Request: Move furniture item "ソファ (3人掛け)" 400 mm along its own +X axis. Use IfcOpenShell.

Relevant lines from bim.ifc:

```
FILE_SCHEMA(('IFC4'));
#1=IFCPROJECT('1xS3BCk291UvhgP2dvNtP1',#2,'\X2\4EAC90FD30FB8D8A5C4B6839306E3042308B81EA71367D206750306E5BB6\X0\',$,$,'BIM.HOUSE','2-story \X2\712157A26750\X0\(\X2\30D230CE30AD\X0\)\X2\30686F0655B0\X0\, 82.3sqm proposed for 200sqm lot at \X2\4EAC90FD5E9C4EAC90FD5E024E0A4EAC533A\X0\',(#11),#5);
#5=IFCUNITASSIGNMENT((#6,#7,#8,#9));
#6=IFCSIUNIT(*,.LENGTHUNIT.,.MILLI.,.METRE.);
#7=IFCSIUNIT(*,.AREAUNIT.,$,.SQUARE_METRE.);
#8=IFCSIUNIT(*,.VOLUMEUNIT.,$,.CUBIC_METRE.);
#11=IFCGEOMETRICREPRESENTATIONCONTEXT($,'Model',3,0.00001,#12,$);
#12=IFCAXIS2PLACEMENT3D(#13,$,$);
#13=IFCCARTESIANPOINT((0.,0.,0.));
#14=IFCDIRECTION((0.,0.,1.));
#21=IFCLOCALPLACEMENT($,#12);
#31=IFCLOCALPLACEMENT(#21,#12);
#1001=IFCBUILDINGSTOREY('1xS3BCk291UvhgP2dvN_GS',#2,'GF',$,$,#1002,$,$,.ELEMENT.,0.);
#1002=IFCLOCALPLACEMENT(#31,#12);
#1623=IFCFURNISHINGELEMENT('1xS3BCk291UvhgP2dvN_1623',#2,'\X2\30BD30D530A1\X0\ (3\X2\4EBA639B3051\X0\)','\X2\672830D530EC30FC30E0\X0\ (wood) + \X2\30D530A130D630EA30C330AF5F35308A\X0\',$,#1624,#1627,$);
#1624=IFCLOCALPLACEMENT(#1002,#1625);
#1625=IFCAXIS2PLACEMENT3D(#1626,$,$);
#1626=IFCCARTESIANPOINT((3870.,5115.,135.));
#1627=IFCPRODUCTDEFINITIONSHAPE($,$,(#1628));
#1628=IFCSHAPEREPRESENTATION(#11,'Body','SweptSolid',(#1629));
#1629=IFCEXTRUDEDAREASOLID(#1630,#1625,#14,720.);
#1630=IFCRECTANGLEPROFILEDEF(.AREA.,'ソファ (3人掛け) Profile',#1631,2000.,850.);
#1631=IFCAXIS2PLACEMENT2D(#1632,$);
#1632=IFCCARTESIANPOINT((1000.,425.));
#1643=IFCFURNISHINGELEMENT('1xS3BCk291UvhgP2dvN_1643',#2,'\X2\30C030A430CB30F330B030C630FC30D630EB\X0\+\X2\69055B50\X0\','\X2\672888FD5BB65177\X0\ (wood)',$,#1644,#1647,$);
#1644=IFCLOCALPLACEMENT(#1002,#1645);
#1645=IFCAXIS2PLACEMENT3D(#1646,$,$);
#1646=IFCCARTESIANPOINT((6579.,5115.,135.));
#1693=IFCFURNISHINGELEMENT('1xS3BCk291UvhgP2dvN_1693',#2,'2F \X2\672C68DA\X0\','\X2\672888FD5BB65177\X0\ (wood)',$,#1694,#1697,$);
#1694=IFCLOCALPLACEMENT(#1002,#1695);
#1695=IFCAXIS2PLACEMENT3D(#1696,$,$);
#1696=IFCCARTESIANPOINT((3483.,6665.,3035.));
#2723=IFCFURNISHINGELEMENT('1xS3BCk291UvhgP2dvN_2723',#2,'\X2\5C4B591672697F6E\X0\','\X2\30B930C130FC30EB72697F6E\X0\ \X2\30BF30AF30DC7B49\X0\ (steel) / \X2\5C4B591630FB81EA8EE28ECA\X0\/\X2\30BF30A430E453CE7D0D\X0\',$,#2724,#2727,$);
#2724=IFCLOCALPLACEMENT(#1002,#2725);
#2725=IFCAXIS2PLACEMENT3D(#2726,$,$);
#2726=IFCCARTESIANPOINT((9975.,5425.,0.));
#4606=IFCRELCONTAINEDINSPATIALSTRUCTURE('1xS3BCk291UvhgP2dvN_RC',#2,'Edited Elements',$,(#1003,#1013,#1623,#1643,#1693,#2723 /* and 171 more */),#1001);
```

```python
import ifcopenshell
import ifcopenshell.api.geometry
import ifcopenshell.util.placement

model = ifcopenshell.open("bim.ifc")

item = model.by_id(1623)
matrix = ifcopenshell.util.placement.get_local_placement(item.ObjectPlacement)
matrix[:3, 3] += matrix[:3, 0] * 400.0
ifcopenshell.api.geometry.edit_object_placement(model, product=item, matrix=matrix, is_si=False)

print(ifcopenshell.util.placement.get_local_placement(item.ObjectPlacement).round(3) + 0.0)

model.write("bim_edited.ifc")
```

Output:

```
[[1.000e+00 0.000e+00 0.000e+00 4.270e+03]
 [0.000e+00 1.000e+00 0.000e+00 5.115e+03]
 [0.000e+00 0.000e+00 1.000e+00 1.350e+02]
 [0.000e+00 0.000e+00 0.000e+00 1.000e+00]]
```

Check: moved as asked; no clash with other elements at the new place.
